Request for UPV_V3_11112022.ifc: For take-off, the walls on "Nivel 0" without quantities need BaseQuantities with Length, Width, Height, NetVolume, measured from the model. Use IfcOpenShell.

First a look at what the model holds.

```python
import ifcopenshell
import ifcopenshell.util.element
import ifcopenshell.util.unit

model = ifcopenshell.open("UPV_V3_11112022.ifc")
print(model.schema)
for unit_type in ("LENGTHUNIT", "AREAUNIT", "VOLUMEUNIT"):
    print(unit_type, ifcopenshell.util.unit.calculate_unit_scale(model, unit_type))
storey = next(s for s in model.by_type("IfcBuildingStorey") if s.Name == "Nivel 0")
walls = [e for e in ifcopenshell.util.element.get_decomposition(storey) if e.is_a("IfcWall")]
for e in sorted(walls, key=lambda e: e.id()):
    print(e.id(), e.is_a(), e.Name, list(ifcopenshell.util.element.get_psets(e, qtos_only=True)), sep=" | ")
```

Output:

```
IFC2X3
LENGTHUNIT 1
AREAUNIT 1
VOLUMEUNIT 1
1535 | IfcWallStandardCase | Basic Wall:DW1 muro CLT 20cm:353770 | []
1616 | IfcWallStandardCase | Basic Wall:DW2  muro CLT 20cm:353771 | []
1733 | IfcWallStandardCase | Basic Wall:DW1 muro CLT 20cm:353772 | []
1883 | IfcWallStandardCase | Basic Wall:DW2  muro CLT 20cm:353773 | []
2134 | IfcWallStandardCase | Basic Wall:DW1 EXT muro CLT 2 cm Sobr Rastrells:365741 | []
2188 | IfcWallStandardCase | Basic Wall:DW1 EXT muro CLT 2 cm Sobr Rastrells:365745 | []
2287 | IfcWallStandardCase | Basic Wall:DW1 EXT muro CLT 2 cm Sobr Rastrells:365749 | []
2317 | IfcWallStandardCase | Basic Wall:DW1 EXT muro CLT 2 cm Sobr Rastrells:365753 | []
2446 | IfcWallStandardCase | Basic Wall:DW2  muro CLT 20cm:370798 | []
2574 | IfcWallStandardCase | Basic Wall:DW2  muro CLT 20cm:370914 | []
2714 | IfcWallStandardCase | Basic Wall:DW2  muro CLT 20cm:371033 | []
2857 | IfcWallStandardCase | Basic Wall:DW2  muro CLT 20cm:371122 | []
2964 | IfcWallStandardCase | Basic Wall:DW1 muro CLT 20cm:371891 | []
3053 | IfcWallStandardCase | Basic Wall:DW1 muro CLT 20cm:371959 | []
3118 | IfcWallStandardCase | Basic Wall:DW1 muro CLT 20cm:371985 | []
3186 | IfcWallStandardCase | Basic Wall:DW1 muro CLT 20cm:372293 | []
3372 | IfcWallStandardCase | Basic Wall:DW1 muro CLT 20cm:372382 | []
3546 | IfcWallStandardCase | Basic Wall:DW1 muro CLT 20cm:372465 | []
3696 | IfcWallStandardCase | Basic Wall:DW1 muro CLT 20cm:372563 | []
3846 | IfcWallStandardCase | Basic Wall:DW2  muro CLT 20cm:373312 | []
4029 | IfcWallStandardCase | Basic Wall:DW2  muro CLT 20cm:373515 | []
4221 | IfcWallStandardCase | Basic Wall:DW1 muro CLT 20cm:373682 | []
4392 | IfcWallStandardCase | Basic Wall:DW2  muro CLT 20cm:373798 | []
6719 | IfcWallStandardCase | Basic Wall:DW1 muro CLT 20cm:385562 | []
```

```python
import ifcopenshell
import ifcopenshell.api.pset
import ifcopenshell.geom
import ifcopenshell.util.element
import ifcopenshell.util.shape
import ifcopenshell.util.unit

model = ifcopenshell.open("UPV_V3_11112022.ifc")
unit_scale = ifcopenshell.util.unit.calculate_unit_scale(model)
volume_scale = ifcopenshell.util.unit.calculate_unit_scale(model, "VOLUMEUNIT")
settings = ifcopenshell.geom.settings()

storey = next(s for s in model.by_type("IfcBuildingStorey") if s.Name == "Nivel 0")
walls = [e for e in ifcopenshell.util.element.get_decomposition(storey) if e.is_a("IfcWall")]

for e in sorted(walls, key=lambda e: e.id()):
    if ifcopenshell.util.element.get_psets(e, qtos_only=True, should_inherit=False):
        continue
    # Geometry comes back in metres, in the element's own axes.
    shape = ifcopenshell.geom.create_shape(settings, e)
    values = {
        "Length": ifcopenshell.util.shape.get_x(shape.geometry) / unit_scale,
        "Width": ifcopenshell.util.shape.get_y(shape.geometry) / unit_scale,
        "Height": ifcopenshell.util.shape.get_z(shape.geometry) / unit_scale,
        "NetVolume": ifcopenshell.util.shape.get_volume(shape.geometry) / volume_scale,
    }
    qto = ifcopenshell.api.pset.add_qto(model, product=e, name="BaseQuantities")
    ifcopenshell.api.pset.edit_qto(model, qto=qto, properties=values)
    print(e.id(), {k: round(v, 3) for k, v in values.items()})

model.write("UPV_V3_11112022_edited.ifc")
```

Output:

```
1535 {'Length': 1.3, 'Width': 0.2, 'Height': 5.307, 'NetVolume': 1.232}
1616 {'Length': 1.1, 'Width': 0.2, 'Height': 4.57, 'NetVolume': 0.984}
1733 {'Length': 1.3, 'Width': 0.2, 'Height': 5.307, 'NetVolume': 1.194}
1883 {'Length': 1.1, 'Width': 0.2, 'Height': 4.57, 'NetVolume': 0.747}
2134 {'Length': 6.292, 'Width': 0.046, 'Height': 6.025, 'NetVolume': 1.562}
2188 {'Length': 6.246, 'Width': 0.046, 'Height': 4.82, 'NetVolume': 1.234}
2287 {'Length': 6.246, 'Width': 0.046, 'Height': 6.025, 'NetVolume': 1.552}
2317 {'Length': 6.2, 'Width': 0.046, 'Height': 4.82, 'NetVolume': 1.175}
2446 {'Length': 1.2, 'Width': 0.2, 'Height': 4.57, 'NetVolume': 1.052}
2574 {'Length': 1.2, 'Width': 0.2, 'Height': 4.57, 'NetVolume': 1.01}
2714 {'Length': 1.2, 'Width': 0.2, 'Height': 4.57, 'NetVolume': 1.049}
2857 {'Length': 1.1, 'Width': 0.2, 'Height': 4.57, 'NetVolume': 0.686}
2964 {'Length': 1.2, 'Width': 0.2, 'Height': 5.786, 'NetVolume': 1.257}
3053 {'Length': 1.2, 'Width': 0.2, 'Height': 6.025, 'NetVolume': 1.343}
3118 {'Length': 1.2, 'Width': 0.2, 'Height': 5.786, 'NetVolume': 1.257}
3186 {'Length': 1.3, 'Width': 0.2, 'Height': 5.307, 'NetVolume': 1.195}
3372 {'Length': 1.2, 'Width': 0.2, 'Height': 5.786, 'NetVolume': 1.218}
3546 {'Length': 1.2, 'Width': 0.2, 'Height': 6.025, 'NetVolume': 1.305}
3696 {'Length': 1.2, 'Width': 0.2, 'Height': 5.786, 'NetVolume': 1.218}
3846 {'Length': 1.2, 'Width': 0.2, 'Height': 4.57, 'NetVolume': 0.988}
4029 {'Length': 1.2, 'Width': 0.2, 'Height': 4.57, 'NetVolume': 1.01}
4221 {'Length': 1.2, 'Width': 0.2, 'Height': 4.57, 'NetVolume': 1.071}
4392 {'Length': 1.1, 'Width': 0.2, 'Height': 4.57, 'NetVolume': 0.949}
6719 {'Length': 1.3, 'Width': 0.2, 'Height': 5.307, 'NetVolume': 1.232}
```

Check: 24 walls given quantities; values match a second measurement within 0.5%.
